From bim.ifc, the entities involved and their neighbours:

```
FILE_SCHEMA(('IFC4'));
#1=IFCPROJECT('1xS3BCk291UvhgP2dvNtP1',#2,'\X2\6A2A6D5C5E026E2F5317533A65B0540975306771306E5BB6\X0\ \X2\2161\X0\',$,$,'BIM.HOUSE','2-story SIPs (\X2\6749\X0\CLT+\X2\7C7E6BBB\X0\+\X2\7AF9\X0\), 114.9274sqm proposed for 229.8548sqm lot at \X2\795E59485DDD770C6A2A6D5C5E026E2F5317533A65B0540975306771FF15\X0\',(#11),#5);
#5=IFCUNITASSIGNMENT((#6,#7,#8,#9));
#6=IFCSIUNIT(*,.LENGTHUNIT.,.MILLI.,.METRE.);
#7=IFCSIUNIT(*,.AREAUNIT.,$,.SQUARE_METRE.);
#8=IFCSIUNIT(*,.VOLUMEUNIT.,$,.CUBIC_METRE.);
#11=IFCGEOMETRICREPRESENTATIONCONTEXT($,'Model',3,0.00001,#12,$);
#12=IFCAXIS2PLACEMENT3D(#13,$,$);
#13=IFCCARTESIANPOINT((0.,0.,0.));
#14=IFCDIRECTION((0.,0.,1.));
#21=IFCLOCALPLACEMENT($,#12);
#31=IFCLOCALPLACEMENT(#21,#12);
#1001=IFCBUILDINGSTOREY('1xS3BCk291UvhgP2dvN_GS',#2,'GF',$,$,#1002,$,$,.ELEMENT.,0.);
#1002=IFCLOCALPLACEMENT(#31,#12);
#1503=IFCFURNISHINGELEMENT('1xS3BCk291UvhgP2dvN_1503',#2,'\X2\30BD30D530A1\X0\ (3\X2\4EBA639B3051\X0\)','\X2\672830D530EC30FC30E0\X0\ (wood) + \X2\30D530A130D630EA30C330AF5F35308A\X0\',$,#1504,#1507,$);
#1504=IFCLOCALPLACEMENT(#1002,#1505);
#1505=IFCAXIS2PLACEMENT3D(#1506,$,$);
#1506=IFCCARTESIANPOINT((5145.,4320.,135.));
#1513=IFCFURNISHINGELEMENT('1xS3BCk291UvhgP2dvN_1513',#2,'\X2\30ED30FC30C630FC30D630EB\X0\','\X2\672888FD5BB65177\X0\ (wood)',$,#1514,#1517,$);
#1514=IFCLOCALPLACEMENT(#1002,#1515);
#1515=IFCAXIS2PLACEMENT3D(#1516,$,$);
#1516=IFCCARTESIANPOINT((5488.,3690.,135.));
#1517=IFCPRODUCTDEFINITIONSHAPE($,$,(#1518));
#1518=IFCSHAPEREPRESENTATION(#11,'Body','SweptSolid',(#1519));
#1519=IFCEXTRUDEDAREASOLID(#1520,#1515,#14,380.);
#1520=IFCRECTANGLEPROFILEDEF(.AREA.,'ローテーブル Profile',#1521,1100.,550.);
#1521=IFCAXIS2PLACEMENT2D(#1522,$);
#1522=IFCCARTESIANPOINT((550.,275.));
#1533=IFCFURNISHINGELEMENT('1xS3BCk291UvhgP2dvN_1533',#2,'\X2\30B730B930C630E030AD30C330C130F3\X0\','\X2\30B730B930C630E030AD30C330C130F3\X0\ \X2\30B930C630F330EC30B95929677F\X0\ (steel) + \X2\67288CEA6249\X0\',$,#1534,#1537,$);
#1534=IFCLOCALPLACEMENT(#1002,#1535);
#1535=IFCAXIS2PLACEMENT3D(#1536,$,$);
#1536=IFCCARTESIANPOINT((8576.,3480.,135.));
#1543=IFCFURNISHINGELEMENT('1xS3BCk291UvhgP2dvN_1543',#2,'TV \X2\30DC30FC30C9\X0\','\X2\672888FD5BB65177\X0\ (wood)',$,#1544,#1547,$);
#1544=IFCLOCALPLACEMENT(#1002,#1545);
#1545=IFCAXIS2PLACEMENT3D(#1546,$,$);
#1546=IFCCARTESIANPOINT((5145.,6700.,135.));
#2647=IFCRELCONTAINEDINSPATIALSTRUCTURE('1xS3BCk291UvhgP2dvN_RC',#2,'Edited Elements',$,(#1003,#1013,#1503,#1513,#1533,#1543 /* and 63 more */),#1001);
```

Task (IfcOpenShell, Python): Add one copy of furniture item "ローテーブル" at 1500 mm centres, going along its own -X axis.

```python
import ifcopenshell
import ifcopenshell.api.geometry
import ifcopenshell.api.root
import ifcopenshell.util.element
import ifcopenshell.util.placement
import ifcopenshell.util.unit

model = ifcopenshell.open("bim.ifc")
unit_scale = ifcopenshell.util.unit.calculate_unit_scale(model)


def reuse_history(source, copy):
    """copy_class also copies each property set's owner history, people and application; keep the originals."""
    for rel in copy.IsDefinedBy:
        if rel.is_a("IfcRelDefinesByProperties") and (history := rel.RelatingPropertyDefinition.OwnerHistory):
            rel.RelatingPropertyDefinition.OwnerHistory = source.OwnerHistory
            ifcopenshell.util.element.remove_deep2(model, history)


source = model.by_guid("1xS3BCk291UvhgP2dvN_1513")
base = ifcopenshell.util.placement.get_local_placement(source.ObjectPlacement)
step = -base[:3, 0] * 1.5 / unit_scale

for i in range(1, 2):
    copy = ifcopenshell.api.root.copy_class(model, product=source)
    copy.Representation = ifcopenshell.util.element.copy_deep(
        model, source.Representation, exclude=["IfcGeometricRepresentationContext", "IfcRepresentationMap"]
    )
    reuse_history(source, copy)
    matrix = base.copy()
    matrix[:3, 3] += i * step
    print("added at", matrix[:3, 3].round(3) + 0.0)
    ifcopenshell.api.geometry.edit_object_placement(model, product=copy, matrix=matrix, is_si=False)

model.write("bim-out.ifc")
```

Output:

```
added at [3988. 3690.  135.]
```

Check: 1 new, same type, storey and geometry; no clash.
